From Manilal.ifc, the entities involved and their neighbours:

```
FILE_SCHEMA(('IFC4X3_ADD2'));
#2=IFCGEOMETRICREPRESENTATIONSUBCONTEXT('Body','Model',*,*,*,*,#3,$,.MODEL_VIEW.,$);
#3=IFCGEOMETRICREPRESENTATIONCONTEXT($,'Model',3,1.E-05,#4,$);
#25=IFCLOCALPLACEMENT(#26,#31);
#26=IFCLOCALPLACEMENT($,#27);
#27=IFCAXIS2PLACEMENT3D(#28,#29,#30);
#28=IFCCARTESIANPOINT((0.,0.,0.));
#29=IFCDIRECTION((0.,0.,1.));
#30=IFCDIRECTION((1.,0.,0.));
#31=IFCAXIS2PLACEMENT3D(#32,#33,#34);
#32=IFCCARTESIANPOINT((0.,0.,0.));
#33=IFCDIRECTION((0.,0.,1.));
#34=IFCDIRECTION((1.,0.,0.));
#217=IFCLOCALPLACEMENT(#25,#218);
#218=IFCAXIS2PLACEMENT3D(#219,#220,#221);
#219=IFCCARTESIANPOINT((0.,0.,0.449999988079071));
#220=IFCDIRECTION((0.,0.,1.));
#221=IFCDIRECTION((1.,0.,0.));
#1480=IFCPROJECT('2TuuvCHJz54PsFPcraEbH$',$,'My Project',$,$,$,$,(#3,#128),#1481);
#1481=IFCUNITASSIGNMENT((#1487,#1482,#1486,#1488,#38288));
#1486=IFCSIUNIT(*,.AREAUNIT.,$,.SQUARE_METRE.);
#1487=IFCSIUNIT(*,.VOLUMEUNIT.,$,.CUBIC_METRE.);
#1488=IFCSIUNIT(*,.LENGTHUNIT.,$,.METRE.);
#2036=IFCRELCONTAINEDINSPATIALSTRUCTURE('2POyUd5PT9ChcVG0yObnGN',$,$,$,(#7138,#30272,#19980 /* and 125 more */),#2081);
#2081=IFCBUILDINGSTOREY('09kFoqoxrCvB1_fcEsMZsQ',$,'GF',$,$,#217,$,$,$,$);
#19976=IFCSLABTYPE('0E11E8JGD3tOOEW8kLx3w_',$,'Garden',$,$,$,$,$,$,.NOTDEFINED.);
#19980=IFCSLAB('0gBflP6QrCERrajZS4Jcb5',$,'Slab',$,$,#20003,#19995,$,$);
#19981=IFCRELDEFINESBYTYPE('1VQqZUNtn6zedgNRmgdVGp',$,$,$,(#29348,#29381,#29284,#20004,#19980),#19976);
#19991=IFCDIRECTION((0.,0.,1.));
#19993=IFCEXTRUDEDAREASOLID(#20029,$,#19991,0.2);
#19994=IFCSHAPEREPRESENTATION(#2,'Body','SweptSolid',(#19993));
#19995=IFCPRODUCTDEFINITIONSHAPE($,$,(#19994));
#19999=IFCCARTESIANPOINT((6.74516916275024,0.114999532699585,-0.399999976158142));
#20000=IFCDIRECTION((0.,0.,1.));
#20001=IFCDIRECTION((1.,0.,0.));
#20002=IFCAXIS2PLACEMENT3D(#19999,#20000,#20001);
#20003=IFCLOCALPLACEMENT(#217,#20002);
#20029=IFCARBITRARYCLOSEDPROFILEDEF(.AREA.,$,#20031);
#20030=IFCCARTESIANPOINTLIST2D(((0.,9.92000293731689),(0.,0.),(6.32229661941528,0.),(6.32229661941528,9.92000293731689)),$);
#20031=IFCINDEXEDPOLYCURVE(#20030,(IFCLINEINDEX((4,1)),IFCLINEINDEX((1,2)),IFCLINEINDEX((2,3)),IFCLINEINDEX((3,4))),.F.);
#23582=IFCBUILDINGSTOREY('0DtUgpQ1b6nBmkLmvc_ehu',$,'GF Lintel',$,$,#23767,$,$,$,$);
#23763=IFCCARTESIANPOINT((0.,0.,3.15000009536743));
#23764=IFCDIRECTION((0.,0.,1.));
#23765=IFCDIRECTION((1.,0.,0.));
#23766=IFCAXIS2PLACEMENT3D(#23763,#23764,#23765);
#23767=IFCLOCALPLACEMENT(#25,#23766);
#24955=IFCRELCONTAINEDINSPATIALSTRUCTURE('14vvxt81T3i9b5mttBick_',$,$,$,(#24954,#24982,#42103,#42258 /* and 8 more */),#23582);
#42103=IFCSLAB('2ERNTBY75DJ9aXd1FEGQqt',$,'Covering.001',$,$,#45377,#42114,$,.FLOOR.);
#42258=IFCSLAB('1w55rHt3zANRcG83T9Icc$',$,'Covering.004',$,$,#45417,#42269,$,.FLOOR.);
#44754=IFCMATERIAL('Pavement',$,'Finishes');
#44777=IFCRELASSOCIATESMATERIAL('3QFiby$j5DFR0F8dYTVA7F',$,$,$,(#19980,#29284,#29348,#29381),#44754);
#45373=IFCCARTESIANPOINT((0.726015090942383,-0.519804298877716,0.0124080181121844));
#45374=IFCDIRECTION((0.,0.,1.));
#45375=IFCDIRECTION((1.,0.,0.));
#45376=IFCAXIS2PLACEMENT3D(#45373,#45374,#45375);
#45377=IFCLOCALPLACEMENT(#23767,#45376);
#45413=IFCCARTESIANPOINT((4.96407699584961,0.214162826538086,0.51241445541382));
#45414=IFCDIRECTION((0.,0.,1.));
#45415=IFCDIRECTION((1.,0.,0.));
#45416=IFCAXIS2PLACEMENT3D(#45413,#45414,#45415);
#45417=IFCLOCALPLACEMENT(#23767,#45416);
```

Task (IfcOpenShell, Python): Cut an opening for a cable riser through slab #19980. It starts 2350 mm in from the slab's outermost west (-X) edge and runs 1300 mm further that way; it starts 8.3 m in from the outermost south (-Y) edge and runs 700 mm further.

```python
import numpy as np
import ifcopenshell
import ifcopenshell.api.feature
import ifcopenshell.api.geometry
import ifcopenshell.api.root
import ifcopenshell.geom
import ifcopenshell.util.placement
import ifcopenshell.util.representation
import ifcopenshell.util.shape
import ifcopenshell.util.unit

model = ifcopenshell.open("Manilal.ifc")
unit_scale = ifcopenshell.util.unit.calculate_unit_scale(model)
settings = ifcopenshell.geom.settings()


def volume(element):
    """Net volume in cubic metres, openings subtracted."""
    shape = ifcopenshell.geom.create_shape(settings, element)
    return ifcopenshell.util.shape.get_volume(shape.geometry)


slab = model.by_id(19980)
before = volume(slab)

# Extent in the slab's own axes, in metres. The edges named are its -X and -Y sides.
slab_shape = ifcopenshell.geom.create_shape(settings, slab)
vertices = ifcopenshell.util.shape.get_vertices(slab_shape.geometry)
x_min, y_min, bottom = vertices.min(axis=0)
top = vertices[:, 2].max()

opening = ifcopenshell.api.root.create_entity(model, ifc_class="IfcOpeningElement", name="Cable riser opening", predefined_type="OPENING")
context = ifcopenshell.util.representation.get_context(model, "Model", "Body", "MODEL_VIEW")
width, depth = 1.3, 0.7
outline = [(0.0, 0.0), (width, 0.0), (width, depth), (0.0, depth), (0.0, 0.0)]
# Overshoot both faces by 50 mm so the cut is clean.
shape = ifcopenshell.api.geometry.add_slab_representation(
    model, context=context, depth=top - bottom + 0.1, polyline=outline
)
ifcopenshell.api.geometry.assign_representation(model, product=opening, representation=shape)

matrix = ifcopenshell.util.placement.get_local_placement(slab.ObjectPlacement)
matrix[:, 3] = matrix @ np.append(np.array([x_min + 2.35, y_min + 8.3, bottom - 0.05]) / unit_scale, 1.0)
ifcopenshell.api.geometry.edit_object_placement(model, product=opening, matrix=matrix, is_si=False)
ifcopenshell.api.feature.add_feature(model, feature=opening, element=slab)

after = volume(slab)

print(f"slab volume {before:.3f} -> {after:.3f} m3")

model.write("Manilal_rev.ifc")
```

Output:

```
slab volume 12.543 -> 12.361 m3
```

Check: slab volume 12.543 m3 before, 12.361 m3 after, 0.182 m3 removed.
